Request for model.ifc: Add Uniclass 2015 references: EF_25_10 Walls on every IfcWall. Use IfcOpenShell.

First a look at what the model holds.

```python
import ifcopenshell

model = ifcopenshell.open("model.ifc")
print(model.schema)
print("classifications:", [c.Name for c in model.by_type("IfcClassification")])
for ifc_class in ("IfcDoor", "IfcRoof", "IfcStair", "IfcWall", "IfcWindow"):
    print(ifc_class, len(model.by_type(ifc_class)))
```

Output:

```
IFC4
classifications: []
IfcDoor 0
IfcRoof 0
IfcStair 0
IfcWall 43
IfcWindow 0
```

```python
import ifcopenshell
import ifcopenshell.api.classification

model = ifcopenshell.open("model.ifc")

system = ifcopenshell.api.classification.add_classification(model, classification="Uniclass 2015")

codes = {
    "IfcWall": ("EF_25_10", "Walls"),
}
for ifc_class, (code, name) in codes.items():
    products = model.by_type(ifc_class)
    ifcopenshell.api.classification.add_reference(
        model, products=products, classification=system, identification=code, name=name
    )
    print(code, len(products))

model.write("model_edited.ifc")
```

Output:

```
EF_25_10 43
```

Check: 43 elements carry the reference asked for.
